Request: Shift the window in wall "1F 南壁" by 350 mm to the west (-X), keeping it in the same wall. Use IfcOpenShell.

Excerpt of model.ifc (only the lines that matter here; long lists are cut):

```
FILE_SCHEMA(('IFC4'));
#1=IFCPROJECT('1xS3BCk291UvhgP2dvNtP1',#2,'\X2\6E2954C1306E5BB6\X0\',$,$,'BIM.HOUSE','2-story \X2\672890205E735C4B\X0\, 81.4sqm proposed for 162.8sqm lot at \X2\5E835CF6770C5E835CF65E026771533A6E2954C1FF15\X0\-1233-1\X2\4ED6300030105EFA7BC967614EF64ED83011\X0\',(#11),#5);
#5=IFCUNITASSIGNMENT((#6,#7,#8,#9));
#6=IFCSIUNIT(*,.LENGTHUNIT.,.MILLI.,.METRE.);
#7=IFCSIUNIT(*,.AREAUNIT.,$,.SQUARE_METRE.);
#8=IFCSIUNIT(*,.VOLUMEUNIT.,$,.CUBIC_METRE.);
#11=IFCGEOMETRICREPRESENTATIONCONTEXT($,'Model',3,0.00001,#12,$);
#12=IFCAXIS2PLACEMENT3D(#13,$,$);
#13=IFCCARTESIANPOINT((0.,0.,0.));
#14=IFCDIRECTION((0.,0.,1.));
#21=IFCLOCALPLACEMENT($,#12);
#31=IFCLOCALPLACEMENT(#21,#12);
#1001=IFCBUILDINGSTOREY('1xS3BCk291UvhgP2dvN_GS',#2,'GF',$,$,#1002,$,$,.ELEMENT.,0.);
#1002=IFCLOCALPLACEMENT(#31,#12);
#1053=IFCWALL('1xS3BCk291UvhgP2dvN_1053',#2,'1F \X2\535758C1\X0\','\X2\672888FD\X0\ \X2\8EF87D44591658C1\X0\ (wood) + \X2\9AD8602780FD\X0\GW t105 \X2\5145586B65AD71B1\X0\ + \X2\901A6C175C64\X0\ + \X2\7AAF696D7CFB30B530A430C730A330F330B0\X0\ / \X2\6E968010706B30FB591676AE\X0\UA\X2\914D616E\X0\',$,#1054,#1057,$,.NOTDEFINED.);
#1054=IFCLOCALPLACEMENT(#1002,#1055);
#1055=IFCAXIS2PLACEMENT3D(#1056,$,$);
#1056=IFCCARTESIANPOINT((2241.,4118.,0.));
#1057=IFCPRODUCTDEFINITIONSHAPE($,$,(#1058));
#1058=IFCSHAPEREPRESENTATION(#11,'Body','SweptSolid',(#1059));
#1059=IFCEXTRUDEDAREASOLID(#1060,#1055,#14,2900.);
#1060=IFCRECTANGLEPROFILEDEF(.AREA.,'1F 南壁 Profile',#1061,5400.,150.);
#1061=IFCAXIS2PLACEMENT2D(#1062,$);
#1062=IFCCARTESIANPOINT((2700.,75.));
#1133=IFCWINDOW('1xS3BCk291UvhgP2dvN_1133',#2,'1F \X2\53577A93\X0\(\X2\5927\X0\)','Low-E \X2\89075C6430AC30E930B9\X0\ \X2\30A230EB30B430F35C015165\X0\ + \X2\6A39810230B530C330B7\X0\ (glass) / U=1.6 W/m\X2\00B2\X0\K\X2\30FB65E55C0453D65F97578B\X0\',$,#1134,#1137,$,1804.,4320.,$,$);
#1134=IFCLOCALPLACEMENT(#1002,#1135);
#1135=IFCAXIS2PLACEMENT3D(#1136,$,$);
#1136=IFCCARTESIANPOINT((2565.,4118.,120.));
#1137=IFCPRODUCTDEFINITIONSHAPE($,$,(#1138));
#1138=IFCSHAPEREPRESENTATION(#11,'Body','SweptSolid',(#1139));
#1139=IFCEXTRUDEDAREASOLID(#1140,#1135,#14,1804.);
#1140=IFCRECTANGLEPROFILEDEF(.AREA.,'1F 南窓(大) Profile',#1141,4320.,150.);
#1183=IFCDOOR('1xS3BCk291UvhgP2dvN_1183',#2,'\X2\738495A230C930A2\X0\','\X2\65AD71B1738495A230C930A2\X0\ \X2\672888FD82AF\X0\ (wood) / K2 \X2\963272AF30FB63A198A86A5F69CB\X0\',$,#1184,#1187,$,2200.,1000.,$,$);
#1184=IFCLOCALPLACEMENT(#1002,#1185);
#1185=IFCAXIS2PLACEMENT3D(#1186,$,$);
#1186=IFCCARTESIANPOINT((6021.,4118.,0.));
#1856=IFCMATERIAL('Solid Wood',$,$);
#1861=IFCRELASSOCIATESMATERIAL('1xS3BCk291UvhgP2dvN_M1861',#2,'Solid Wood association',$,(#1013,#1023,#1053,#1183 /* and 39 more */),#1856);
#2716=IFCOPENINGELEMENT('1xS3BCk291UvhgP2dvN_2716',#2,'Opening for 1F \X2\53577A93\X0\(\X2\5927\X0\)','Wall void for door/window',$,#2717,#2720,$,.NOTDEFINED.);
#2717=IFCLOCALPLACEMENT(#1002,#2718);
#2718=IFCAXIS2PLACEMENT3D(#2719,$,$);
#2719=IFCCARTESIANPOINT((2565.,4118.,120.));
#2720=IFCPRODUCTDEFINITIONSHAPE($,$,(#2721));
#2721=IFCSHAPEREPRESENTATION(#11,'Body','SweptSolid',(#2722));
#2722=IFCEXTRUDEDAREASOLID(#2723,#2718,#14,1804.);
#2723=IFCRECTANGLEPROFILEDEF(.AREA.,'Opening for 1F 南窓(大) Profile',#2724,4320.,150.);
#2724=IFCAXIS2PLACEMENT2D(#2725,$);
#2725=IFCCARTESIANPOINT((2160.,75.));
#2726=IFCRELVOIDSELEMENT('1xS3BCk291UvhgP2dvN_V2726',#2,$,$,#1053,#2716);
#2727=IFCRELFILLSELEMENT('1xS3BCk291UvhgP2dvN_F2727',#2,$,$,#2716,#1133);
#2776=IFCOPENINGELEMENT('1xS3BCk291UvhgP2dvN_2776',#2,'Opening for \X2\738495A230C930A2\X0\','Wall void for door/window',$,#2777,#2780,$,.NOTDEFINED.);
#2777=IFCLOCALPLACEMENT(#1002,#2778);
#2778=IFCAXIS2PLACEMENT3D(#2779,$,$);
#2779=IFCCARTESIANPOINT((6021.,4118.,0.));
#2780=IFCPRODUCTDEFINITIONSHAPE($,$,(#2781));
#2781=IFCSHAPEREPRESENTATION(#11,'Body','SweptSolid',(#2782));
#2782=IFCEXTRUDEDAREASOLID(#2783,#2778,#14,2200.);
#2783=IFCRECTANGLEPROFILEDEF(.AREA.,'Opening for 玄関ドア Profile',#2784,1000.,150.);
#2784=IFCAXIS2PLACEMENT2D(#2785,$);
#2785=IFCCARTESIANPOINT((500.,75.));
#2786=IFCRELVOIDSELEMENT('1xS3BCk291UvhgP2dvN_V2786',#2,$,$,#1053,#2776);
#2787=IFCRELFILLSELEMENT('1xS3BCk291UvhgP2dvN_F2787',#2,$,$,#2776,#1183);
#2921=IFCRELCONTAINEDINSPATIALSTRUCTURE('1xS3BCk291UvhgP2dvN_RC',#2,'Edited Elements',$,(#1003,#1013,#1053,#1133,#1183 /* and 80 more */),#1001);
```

```python
import ifcopenshell
import ifcopenshell.api.geometry
import ifcopenshell.util.placement
import ifcopenshell.util.unit

model = ifcopenshell.open("model.ifc")
unit_scale = ifcopenshell.util.unit.calculate_unit_scale(model)

window = model.by_guid("1xS3BCk291UvhgP2dvN_1133")
opening = window.FillsVoids[0].RelatingOpeningElement
wall = opening.VoidsElements[0].RelatingBuildingElement

wall_matrix = ifcopenshell.util.placement.get_local_placement(wall.ObjectPlacement)
shift = wall_matrix[:3, 0] * -0.35 / unit_scale
before = ifcopenshell.util.placement.get_local_placement(window.ObjectPlacement)[:3, 3].copy()

# The window is not placed relative to its opening, so move both.
for product in (opening, window):
    matrix = ifcopenshell.util.placement.get_local_placement(product.ObjectPlacement)
    matrix[:3, 3] += shift
    ifcopenshell.api.geometry.edit_object_placement(model, product=product, matrix=matrix, is_si=False)

after = ifcopenshell.util.placement.get_local_placement(window.ObjectPlacement)[:3, 3]
print("window moved by", (after - before).round(3) + 0.0)

model.write("model-out.ifc")
```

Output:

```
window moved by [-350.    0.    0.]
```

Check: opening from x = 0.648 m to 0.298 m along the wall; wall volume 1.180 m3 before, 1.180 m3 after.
